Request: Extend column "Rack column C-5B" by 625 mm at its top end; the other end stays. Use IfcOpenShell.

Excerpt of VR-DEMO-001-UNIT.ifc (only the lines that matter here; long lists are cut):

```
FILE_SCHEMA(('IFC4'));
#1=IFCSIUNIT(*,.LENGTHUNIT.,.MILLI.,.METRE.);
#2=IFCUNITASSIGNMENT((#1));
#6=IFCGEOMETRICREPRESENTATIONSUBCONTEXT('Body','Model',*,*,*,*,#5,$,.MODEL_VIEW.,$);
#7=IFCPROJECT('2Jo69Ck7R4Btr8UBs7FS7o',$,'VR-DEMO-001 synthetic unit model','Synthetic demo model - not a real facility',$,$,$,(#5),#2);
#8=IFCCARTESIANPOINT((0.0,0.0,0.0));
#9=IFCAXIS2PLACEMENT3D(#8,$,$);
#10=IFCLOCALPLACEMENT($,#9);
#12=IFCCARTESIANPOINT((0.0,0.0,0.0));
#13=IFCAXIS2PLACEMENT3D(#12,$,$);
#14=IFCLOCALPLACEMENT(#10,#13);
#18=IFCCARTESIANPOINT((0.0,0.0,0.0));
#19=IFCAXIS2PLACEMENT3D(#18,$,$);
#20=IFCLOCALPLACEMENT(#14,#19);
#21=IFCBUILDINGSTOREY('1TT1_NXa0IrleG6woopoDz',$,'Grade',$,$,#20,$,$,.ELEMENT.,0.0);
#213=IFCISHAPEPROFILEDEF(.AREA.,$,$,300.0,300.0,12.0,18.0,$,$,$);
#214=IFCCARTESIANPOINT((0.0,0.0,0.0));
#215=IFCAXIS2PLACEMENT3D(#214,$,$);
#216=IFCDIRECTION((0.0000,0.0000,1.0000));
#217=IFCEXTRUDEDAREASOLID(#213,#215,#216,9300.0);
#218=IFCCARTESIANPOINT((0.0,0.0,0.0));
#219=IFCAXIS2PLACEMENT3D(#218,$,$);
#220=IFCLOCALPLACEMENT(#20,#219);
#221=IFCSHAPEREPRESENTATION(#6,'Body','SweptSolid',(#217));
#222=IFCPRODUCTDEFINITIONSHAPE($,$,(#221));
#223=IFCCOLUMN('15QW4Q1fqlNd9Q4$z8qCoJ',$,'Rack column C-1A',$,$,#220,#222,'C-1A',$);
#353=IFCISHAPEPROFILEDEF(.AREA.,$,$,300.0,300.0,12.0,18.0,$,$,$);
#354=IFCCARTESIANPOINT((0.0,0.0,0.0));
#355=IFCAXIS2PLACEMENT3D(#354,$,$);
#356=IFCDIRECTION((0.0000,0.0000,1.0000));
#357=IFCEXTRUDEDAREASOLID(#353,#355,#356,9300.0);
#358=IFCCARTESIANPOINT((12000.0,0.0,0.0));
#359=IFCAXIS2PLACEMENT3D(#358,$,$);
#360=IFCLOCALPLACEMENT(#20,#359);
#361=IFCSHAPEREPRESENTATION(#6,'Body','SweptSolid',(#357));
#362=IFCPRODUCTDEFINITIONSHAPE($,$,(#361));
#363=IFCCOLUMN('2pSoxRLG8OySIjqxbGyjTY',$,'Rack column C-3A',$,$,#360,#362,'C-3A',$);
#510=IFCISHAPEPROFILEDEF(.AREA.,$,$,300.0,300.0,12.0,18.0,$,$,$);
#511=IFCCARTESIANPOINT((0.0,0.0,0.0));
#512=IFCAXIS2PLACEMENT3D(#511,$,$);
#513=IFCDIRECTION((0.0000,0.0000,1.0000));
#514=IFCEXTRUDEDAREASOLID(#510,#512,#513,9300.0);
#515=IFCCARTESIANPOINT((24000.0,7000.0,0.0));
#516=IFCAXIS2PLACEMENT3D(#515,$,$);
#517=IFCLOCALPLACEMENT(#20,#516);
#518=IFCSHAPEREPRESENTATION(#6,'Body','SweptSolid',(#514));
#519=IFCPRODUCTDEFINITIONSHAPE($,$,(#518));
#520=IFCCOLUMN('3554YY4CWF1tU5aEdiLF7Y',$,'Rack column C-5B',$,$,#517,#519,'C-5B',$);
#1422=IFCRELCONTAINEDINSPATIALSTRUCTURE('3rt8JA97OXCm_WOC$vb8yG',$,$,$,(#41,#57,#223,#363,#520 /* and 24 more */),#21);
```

```python
import ifcopenshell
import ifcopenshell.util.representation
import ifcopenshell.util.unit

model = ifcopenshell.open("VR-DEMO-001-UNIT.ifc")
unit_scale = ifcopenshell.util.unit.calculate_unit_scale(model)

member = model.by_id(520)
change = 0.625 / unit_scale

# The extrusion runs towards the end named, so only its depth changes.
body = ifcopenshell.util.representation.get_representation(member, "Model", "Body")
solid = body.Items[0]
old_length = solid.Depth
solid.Depth += change

print(f"length {old_length:g} -> {solid.Depth:g}")

model.write("VR-DEMO-001-UNIT_rev.ifc")
```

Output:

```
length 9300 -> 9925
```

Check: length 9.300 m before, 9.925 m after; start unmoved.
